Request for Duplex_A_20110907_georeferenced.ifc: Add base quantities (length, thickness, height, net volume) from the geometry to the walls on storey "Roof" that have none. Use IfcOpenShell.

First a look at what the model holds.

```python
import ifcopenshell
import ifcopenshell.util.element
import ifcopenshell.util.unit

model = ifcopenshell.open("Duplex_A_20110907_georeferenced.ifc")
print(model.schema)
for unit_type in ("LENGTHUNIT", "AREAUNIT", "VOLUMEUNIT"):
    print(unit_type, ifcopenshell.util.unit.calculate_unit_scale(model, unit_type))
storey = next(s for s in model.by_type("IfcBuildingStorey") if s.Name == "Roof")
walls = [e for e in ifcopenshell.util.element.get_decomposition(storey) if e.is_a("IfcWall")]
for e in sorted(walls, key=lambda e: e.id()):
    print(e.id(), e.is_a(), e.Name, list(ifcopenshell.util.element.get_psets(e, qtos_only=True)), sep=" | ")
```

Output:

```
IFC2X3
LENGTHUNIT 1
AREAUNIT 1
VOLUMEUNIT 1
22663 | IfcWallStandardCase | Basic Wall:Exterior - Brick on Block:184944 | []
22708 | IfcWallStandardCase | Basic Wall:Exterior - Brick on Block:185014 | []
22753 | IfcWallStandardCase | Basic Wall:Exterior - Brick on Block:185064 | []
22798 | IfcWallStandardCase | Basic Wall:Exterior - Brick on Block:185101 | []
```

```python
import ifcopenshell
import ifcopenshell.api.pset
import ifcopenshell.geom
import ifcopenshell.util.element
import ifcopenshell.util.shape
import ifcopenshell.util.unit

model = ifcopenshell.open("Duplex_A_20110907_georeferenced.ifc")
unit_scale = ifcopenshell.util.unit.calculate_unit_scale(model)
volume_scale = ifcopenshell.util.unit.calculate_unit_scale(model, "VOLUMEUNIT")
settings = ifcopenshell.geom.settings()

storey = next(s for s in model.by_type("IfcBuildingStorey") if s.Name == "Roof")
walls = [e for e in ifcopenshell.util.element.get_decomposition(storey) if e.is_a("IfcWall")]

for e in sorted(walls, key=lambda e: e.id()):
    if ifcopenshell.util.element.get_psets(e, qtos_only=True, should_inherit=False):
        continue
    # Geometry comes back in metres, in the element's own axes.
    shape = ifcopenshell.geom.create_shape(settings, e)
    values = {
        "Length": ifcopenshell.util.shape.get_x(shape.geometry) / unit_scale,
        "Width": ifcopenshell.util.shape.get_y(shape.geometry) / unit_scale,
        "Height": ifcopenshell.util.shape.get_z(shape.geometry) / unit_scale,
        "NetVolume": ifcopenshell.util.shape.get_volume(shape.geometry) / volume_scale,
    }
    qto = ifcopenshell.api.pset.add_qto(model, product=e, name="BaseQuantities")
    ifcopenshell.api.pset.edit_qto(model, qto=qto, properties=values)
    print(e.id(), {k: round(v, 3) for k, v in values.items()})

model.write("Duplex_A_20110907_georeferenced_rev.ifc")
```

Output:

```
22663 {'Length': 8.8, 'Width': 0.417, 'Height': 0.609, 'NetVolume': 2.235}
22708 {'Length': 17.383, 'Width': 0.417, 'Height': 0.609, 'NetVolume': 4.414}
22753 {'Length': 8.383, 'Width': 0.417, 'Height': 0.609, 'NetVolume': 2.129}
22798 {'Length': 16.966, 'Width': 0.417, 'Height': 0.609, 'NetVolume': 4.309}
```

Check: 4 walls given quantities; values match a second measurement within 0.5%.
